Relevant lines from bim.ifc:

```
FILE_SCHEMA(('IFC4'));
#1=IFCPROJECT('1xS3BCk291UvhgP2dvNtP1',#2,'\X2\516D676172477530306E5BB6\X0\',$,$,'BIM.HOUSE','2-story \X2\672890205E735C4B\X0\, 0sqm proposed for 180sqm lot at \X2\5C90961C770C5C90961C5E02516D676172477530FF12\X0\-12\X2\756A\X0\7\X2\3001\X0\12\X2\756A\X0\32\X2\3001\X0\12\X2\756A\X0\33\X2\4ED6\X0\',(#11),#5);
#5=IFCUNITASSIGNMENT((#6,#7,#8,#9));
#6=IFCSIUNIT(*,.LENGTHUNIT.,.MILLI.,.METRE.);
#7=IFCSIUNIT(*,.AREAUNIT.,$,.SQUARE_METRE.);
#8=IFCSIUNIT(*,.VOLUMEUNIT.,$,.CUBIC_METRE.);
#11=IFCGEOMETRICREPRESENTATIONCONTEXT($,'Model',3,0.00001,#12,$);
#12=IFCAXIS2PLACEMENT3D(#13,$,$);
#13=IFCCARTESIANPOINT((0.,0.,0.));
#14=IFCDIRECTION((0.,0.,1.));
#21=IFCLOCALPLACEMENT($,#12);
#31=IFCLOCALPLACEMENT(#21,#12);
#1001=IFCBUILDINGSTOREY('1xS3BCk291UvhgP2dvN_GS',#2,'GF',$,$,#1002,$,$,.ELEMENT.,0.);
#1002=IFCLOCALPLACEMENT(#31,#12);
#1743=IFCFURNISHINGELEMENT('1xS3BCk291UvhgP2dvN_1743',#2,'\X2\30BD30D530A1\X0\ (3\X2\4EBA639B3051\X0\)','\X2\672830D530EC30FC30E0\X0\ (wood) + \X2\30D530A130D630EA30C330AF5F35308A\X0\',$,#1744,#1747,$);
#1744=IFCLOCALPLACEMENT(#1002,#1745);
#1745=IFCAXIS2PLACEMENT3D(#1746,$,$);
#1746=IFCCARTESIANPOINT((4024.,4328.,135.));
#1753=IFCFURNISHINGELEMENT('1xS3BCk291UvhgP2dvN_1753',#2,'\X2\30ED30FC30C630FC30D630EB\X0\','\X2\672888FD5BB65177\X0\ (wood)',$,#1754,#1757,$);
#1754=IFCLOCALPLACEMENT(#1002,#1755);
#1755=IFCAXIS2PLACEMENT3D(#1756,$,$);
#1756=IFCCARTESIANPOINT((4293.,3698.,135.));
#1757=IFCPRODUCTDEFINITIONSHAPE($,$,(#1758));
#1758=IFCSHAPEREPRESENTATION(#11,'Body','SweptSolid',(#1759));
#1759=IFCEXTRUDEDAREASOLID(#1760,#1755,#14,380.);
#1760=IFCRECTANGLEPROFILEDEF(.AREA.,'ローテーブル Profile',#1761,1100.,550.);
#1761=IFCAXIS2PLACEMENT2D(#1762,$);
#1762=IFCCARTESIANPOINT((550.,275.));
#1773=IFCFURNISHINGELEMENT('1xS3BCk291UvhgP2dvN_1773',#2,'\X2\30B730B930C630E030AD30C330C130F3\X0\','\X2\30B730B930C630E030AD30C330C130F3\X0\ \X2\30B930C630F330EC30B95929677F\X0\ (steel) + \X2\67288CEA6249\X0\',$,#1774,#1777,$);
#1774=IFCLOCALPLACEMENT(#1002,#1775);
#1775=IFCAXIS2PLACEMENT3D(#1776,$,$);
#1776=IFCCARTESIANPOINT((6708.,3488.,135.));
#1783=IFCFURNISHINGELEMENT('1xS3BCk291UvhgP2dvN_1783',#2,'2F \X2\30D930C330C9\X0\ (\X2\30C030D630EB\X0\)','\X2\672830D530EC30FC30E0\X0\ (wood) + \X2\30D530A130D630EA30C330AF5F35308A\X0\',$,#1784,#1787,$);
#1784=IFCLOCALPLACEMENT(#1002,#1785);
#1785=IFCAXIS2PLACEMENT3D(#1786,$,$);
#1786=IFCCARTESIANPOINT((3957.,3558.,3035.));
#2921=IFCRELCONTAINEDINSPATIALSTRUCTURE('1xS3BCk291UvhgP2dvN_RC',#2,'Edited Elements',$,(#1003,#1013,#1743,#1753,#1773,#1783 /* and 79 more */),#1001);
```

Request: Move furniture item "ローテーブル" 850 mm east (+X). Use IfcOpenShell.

```python
import ifcopenshell
import ifcopenshell.api.geometry
import ifcopenshell.util.placement
import ifcopenshell.util.unit

model = ifcopenshell.open("bim.ifc")
unit_scale = ifcopenshell.util.unit.calculate_unit_scale(model)

item = model.by_guid("1xS3BCk291UvhgP2dvN_1753")
matrix = ifcopenshell.util.placement.get_local_placement(item.ObjectPlacement)
matrix[0, 3] += 0.85 / unit_scale
ifcopenshell.api.geometry.edit_object_placement(model, product=item, matrix=matrix, is_si=False)

print(ifcopenshell.util.placement.get_local_placement(item.ObjectPlacement).round(3) + 0.0)

model.write("bim-out.ifc")
```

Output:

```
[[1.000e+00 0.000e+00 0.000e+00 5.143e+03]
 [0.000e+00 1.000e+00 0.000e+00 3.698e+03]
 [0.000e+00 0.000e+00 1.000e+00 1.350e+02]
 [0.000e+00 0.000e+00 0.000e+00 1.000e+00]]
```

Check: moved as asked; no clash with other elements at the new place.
